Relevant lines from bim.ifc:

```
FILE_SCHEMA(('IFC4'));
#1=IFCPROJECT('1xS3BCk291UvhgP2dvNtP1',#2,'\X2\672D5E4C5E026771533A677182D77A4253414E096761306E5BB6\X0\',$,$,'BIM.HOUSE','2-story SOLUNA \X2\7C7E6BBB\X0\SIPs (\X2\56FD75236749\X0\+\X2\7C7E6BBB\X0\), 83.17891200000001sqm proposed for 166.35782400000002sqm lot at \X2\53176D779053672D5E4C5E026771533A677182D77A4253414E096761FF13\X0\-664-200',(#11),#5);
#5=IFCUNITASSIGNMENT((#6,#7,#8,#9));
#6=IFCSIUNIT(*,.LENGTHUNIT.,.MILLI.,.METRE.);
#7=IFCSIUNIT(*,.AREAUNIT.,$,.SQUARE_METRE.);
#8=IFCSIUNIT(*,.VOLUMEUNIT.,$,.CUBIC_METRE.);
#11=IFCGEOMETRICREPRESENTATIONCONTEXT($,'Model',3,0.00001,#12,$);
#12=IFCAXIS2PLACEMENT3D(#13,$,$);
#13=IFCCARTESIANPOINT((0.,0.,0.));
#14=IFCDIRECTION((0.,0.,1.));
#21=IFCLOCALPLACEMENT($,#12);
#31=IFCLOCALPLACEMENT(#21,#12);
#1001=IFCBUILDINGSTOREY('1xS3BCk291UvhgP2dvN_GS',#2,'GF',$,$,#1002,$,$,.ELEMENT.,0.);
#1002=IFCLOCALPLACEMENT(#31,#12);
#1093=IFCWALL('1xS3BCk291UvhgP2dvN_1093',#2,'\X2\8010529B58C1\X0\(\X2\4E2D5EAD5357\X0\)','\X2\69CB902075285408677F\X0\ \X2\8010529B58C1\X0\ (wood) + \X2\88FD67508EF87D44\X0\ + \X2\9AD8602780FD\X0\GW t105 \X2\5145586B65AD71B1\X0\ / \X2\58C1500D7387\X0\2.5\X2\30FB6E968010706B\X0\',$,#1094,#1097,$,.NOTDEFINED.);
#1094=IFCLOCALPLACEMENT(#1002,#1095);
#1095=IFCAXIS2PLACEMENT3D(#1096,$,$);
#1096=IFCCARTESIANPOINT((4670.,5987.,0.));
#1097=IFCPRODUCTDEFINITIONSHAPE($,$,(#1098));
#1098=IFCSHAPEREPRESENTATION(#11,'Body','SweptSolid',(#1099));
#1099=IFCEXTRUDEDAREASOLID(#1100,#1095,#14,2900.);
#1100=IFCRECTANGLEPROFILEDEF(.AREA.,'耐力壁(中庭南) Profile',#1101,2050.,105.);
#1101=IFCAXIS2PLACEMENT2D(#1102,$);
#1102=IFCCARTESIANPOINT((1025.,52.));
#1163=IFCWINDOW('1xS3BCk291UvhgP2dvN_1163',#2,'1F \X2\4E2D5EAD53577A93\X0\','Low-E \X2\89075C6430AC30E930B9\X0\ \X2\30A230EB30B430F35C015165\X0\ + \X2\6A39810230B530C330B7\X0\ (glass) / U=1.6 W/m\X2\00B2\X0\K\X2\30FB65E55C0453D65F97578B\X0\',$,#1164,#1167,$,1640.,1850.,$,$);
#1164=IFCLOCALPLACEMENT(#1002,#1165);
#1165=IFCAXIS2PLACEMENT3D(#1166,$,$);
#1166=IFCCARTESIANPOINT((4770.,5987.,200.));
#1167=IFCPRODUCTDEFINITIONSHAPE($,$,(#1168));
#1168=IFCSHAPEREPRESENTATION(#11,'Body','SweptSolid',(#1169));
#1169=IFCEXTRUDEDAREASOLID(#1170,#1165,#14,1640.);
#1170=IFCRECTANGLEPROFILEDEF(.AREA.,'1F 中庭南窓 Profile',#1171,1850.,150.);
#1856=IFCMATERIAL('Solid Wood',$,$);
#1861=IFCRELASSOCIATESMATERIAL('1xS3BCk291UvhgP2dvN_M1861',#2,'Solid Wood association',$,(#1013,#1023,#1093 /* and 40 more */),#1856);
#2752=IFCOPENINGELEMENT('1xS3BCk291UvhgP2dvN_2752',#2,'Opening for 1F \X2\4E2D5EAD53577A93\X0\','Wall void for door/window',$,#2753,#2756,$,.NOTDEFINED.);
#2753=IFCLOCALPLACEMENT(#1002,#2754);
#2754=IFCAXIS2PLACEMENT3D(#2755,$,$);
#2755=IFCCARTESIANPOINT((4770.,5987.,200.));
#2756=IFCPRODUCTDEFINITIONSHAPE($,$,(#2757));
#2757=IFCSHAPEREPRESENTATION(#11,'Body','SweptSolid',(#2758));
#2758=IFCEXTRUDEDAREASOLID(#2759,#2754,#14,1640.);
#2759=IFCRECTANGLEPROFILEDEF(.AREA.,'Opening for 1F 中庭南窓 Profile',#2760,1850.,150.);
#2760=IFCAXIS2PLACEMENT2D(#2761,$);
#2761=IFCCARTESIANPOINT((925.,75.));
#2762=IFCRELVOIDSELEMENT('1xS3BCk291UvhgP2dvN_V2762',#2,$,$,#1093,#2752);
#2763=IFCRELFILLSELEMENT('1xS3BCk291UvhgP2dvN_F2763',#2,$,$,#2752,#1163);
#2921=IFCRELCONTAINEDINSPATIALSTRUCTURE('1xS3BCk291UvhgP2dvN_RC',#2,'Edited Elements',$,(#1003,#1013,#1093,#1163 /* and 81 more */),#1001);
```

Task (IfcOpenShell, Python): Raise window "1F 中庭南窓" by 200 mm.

```python
import numpy as np
import ifcopenshell
import ifcopenshell.api.geometry
import ifcopenshell.util.placement
import ifcopenshell.util.unit

model = ifcopenshell.open("bim.ifc")
unit_scale = ifcopenshell.util.unit.calculate_unit_scale(model)

window = model.by_guid("1xS3BCk291UvhgP2dvN_1163")
opening = window.FillsVoids[0].RelatingOpeningElement
dz = 0.2 / unit_scale

shift = np.array([0.0, 0.0, dz])
# The window is not placed relative to its opening, so move both.
for product in (opening, window):
    matrix = ifcopenshell.util.placement.get_local_placement(product.ObjectPlacement)
    matrix[:3, 3] += shift
    ifcopenshell.api.geometry.edit_object_placement(model, product=product, matrix=matrix, is_si=False)

print(f"moved by {dz * unit_scale:+.3f} m")

model.write("bim-out.ifc")
```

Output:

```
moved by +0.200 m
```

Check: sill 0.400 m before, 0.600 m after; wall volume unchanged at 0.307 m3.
